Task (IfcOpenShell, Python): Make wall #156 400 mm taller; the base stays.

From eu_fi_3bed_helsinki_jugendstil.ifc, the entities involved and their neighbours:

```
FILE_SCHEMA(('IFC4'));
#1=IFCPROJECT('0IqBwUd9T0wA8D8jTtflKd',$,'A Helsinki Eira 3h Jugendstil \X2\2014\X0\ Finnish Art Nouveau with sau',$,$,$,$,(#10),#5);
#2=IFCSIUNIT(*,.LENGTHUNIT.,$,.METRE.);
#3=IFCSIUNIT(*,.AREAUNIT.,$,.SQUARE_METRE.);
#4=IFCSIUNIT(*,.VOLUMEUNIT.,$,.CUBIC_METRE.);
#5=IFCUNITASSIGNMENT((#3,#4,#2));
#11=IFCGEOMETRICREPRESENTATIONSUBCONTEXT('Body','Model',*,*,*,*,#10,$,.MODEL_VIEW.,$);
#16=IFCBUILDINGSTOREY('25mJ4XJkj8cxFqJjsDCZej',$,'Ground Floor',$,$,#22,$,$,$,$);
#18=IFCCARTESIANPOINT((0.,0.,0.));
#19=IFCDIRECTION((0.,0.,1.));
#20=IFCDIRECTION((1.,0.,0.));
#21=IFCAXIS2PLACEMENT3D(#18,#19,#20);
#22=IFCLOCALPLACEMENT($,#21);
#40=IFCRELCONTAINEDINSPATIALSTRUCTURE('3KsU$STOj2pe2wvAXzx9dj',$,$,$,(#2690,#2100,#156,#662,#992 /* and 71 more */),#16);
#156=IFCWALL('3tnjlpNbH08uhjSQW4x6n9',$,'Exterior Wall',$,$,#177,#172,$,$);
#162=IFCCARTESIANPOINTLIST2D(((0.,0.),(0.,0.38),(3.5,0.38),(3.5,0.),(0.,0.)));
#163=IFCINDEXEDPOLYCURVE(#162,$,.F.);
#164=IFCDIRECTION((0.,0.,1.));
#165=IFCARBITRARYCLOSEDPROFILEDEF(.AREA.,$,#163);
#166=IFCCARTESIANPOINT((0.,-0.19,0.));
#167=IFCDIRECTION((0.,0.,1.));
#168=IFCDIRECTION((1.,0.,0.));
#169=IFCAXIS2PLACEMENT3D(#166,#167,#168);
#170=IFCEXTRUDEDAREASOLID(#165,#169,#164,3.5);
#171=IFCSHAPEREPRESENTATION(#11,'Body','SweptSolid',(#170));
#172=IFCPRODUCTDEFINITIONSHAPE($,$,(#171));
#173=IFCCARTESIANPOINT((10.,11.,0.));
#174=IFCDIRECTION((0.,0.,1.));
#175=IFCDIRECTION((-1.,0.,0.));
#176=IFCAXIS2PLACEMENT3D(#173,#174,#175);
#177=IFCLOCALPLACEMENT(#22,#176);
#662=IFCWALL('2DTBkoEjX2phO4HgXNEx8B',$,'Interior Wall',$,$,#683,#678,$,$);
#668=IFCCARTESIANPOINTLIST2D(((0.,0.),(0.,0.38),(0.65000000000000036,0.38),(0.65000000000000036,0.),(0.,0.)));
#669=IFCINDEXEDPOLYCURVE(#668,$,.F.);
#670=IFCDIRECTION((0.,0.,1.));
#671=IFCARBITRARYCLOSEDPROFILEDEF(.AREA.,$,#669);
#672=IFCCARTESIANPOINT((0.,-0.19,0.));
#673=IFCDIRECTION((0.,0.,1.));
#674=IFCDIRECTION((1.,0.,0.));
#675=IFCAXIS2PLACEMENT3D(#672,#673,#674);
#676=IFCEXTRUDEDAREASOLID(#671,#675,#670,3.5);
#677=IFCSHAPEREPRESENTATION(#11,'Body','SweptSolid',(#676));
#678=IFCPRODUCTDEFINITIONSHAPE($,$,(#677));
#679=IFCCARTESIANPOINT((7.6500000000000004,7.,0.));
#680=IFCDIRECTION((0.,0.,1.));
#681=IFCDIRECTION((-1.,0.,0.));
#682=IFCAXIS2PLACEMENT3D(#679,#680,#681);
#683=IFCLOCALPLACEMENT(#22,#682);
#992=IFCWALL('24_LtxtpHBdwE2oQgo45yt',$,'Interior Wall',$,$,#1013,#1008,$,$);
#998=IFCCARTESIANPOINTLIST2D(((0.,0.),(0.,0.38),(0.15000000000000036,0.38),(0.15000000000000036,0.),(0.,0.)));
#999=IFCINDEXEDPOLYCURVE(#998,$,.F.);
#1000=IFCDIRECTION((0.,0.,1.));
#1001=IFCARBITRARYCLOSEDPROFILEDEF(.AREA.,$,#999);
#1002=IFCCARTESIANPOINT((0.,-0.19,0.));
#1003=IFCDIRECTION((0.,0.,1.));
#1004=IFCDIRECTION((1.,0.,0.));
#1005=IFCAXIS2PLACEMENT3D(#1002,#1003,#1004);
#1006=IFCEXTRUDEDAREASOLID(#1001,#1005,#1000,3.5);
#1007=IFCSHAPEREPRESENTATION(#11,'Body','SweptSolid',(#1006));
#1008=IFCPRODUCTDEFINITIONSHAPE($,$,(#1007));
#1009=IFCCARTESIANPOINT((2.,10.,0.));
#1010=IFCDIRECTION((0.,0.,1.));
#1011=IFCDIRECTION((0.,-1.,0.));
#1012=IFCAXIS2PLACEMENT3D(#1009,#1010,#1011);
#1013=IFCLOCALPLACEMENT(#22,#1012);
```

```python
import ifcopenshell
import ifcopenshell.geom
import ifcopenshell.util.representation
import ifcopenshell.util.shape
import ifcopenshell.util.unit

model = ifcopenshell.open("eu_fi_3bed_helsinki_jugendstil.ifc")
unit_scale = ifcopenshell.util.unit.calculate_unit_scale(model)
settings = ifcopenshell.geom.settings()


def volume(element):
    """Net volume in cubic metres, openings subtracted."""
    shape = ifcopenshell.geom.create_shape(settings, element)
    return ifcopenshell.util.shape.get_volume(shape.geometry)


wall = model.by_guid("3tnjlpNbH08uhjSQW4x6n9")
before = volume(wall)

body = ifcopenshell.util.representation.get_representation(wall, "Model", "Body")
solid = body.Items[0]
old_height = solid.Depth
solid.Depth += 0.4 / unit_scale
after = volume(wall)

print(f"height {old_height:g} -> {solid.Depth:g}, volume {before:.3f} -> {after:.3f} m3")

model.write("eu_fi_3bed_helsinki_jugendstil-out.ifc")
```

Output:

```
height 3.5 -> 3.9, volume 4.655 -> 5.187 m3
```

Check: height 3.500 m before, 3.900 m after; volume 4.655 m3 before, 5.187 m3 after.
